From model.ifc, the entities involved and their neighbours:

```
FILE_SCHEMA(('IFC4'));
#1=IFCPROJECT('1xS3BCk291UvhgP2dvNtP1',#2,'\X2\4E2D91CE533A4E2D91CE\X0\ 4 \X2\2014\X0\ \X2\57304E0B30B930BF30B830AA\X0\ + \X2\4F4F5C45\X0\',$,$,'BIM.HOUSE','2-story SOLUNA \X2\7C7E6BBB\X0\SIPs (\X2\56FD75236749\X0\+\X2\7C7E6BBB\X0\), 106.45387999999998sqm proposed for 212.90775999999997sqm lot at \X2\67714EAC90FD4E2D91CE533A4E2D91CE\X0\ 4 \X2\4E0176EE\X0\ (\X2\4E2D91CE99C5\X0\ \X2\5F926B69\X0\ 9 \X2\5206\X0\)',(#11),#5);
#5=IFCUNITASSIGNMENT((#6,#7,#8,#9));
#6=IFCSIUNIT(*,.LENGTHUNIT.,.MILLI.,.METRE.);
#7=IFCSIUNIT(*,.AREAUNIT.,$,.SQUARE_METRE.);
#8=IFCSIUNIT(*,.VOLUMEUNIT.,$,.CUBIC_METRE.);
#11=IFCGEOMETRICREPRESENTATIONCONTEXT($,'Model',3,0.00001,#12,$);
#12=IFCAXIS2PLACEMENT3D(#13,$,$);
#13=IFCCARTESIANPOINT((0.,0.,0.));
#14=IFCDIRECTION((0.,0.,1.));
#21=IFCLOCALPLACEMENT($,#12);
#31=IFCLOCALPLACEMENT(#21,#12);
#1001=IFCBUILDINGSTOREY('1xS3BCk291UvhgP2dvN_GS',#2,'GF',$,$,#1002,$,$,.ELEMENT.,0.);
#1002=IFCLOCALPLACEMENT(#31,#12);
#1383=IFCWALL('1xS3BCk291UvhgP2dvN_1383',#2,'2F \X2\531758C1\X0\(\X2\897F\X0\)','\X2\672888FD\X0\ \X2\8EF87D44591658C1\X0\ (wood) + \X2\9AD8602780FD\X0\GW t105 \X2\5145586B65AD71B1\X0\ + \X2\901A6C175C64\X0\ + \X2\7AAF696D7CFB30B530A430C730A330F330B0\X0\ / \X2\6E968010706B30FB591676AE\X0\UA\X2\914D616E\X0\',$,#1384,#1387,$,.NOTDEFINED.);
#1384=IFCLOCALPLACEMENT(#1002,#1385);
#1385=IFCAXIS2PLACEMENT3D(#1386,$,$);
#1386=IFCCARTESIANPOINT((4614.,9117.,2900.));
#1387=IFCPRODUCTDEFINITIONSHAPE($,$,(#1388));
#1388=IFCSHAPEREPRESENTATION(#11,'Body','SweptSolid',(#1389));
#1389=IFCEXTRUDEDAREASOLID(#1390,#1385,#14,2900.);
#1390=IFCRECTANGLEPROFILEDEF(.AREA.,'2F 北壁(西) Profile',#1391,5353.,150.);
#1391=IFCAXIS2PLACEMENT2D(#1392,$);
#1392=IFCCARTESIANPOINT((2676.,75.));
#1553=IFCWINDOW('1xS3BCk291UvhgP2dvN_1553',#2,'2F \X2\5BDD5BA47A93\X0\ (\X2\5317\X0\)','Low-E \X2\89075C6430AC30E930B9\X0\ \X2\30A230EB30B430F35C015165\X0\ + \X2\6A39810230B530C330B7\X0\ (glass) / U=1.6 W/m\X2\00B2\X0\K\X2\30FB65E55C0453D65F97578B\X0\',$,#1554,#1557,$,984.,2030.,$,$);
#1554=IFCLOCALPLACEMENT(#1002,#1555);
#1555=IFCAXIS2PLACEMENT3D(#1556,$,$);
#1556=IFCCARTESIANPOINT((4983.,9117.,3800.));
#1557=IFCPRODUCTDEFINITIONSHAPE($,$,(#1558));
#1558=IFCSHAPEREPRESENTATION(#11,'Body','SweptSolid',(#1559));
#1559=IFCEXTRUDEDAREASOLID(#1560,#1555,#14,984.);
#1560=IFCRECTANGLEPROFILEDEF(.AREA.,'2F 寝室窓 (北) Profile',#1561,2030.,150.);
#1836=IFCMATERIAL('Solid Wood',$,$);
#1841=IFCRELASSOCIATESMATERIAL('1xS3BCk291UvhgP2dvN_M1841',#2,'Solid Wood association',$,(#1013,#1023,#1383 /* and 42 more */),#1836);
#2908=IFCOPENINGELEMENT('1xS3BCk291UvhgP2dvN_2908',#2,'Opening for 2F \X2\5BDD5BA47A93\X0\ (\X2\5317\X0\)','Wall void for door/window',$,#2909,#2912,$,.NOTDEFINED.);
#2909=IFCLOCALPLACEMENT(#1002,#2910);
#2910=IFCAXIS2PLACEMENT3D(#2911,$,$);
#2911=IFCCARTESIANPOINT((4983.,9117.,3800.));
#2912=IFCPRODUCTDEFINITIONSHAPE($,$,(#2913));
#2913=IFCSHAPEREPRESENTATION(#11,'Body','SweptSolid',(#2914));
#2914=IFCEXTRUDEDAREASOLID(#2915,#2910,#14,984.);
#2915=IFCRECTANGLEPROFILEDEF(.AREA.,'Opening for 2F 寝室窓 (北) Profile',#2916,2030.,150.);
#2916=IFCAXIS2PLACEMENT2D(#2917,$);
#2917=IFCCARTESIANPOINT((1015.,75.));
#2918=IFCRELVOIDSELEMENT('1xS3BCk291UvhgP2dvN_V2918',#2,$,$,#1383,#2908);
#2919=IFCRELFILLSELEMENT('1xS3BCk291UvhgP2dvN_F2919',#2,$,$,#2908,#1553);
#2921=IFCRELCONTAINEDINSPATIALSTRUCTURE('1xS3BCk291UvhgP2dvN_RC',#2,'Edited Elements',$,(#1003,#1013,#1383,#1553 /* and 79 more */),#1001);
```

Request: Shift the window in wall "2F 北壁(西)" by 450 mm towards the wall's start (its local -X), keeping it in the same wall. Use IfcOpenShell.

```python
import ifcopenshell
import ifcopenshell.api.geometry
import ifcopenshell.util.placement
import ifcopenshell.util.unit

model = ifcopenshell.open("model.ifc")
unit_scale = ifcopenshell.util.unit.calculate_unit_scale(model)

window = model.by_guid("1xS3BCk291UvhgP2dvN_1553")
opening = window.FillsVoids[0].RelatingOpeningElement
wall = opening.VoidsElements[0].RelatingBuildingElement

wall_matrix = ifcopenshell.util.placement.get_local_placement(wall.ObjectPlacement)
shift = wall_matrix[:3, 0] * -0.45 / unit_scale
before = ifcopenshell.util.placement.get_local_placement(window.ObjectPlacement)[:3, 3].copy()

# The window is not placed relative to its opening, so move both.
for product in (opening, window):
    matrix = ifcopenshell.util.placement.get_local_placement(product.ObjectPlacement)
    matrix[:3, 3] += shift
    ifcopenshell.api.geometry.edit_object_placement(model, product=product, matrix=matrix, is_si=False)

after = ifcopenshell.util.placement.get_local_placement(window.ObjectPlacement)[:3, 3]
print("window moved by", (after - before).round(3) + 0.0)

model.write("model_edited.ifc")
```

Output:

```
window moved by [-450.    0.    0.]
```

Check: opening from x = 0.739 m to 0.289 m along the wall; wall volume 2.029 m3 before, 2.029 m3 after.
